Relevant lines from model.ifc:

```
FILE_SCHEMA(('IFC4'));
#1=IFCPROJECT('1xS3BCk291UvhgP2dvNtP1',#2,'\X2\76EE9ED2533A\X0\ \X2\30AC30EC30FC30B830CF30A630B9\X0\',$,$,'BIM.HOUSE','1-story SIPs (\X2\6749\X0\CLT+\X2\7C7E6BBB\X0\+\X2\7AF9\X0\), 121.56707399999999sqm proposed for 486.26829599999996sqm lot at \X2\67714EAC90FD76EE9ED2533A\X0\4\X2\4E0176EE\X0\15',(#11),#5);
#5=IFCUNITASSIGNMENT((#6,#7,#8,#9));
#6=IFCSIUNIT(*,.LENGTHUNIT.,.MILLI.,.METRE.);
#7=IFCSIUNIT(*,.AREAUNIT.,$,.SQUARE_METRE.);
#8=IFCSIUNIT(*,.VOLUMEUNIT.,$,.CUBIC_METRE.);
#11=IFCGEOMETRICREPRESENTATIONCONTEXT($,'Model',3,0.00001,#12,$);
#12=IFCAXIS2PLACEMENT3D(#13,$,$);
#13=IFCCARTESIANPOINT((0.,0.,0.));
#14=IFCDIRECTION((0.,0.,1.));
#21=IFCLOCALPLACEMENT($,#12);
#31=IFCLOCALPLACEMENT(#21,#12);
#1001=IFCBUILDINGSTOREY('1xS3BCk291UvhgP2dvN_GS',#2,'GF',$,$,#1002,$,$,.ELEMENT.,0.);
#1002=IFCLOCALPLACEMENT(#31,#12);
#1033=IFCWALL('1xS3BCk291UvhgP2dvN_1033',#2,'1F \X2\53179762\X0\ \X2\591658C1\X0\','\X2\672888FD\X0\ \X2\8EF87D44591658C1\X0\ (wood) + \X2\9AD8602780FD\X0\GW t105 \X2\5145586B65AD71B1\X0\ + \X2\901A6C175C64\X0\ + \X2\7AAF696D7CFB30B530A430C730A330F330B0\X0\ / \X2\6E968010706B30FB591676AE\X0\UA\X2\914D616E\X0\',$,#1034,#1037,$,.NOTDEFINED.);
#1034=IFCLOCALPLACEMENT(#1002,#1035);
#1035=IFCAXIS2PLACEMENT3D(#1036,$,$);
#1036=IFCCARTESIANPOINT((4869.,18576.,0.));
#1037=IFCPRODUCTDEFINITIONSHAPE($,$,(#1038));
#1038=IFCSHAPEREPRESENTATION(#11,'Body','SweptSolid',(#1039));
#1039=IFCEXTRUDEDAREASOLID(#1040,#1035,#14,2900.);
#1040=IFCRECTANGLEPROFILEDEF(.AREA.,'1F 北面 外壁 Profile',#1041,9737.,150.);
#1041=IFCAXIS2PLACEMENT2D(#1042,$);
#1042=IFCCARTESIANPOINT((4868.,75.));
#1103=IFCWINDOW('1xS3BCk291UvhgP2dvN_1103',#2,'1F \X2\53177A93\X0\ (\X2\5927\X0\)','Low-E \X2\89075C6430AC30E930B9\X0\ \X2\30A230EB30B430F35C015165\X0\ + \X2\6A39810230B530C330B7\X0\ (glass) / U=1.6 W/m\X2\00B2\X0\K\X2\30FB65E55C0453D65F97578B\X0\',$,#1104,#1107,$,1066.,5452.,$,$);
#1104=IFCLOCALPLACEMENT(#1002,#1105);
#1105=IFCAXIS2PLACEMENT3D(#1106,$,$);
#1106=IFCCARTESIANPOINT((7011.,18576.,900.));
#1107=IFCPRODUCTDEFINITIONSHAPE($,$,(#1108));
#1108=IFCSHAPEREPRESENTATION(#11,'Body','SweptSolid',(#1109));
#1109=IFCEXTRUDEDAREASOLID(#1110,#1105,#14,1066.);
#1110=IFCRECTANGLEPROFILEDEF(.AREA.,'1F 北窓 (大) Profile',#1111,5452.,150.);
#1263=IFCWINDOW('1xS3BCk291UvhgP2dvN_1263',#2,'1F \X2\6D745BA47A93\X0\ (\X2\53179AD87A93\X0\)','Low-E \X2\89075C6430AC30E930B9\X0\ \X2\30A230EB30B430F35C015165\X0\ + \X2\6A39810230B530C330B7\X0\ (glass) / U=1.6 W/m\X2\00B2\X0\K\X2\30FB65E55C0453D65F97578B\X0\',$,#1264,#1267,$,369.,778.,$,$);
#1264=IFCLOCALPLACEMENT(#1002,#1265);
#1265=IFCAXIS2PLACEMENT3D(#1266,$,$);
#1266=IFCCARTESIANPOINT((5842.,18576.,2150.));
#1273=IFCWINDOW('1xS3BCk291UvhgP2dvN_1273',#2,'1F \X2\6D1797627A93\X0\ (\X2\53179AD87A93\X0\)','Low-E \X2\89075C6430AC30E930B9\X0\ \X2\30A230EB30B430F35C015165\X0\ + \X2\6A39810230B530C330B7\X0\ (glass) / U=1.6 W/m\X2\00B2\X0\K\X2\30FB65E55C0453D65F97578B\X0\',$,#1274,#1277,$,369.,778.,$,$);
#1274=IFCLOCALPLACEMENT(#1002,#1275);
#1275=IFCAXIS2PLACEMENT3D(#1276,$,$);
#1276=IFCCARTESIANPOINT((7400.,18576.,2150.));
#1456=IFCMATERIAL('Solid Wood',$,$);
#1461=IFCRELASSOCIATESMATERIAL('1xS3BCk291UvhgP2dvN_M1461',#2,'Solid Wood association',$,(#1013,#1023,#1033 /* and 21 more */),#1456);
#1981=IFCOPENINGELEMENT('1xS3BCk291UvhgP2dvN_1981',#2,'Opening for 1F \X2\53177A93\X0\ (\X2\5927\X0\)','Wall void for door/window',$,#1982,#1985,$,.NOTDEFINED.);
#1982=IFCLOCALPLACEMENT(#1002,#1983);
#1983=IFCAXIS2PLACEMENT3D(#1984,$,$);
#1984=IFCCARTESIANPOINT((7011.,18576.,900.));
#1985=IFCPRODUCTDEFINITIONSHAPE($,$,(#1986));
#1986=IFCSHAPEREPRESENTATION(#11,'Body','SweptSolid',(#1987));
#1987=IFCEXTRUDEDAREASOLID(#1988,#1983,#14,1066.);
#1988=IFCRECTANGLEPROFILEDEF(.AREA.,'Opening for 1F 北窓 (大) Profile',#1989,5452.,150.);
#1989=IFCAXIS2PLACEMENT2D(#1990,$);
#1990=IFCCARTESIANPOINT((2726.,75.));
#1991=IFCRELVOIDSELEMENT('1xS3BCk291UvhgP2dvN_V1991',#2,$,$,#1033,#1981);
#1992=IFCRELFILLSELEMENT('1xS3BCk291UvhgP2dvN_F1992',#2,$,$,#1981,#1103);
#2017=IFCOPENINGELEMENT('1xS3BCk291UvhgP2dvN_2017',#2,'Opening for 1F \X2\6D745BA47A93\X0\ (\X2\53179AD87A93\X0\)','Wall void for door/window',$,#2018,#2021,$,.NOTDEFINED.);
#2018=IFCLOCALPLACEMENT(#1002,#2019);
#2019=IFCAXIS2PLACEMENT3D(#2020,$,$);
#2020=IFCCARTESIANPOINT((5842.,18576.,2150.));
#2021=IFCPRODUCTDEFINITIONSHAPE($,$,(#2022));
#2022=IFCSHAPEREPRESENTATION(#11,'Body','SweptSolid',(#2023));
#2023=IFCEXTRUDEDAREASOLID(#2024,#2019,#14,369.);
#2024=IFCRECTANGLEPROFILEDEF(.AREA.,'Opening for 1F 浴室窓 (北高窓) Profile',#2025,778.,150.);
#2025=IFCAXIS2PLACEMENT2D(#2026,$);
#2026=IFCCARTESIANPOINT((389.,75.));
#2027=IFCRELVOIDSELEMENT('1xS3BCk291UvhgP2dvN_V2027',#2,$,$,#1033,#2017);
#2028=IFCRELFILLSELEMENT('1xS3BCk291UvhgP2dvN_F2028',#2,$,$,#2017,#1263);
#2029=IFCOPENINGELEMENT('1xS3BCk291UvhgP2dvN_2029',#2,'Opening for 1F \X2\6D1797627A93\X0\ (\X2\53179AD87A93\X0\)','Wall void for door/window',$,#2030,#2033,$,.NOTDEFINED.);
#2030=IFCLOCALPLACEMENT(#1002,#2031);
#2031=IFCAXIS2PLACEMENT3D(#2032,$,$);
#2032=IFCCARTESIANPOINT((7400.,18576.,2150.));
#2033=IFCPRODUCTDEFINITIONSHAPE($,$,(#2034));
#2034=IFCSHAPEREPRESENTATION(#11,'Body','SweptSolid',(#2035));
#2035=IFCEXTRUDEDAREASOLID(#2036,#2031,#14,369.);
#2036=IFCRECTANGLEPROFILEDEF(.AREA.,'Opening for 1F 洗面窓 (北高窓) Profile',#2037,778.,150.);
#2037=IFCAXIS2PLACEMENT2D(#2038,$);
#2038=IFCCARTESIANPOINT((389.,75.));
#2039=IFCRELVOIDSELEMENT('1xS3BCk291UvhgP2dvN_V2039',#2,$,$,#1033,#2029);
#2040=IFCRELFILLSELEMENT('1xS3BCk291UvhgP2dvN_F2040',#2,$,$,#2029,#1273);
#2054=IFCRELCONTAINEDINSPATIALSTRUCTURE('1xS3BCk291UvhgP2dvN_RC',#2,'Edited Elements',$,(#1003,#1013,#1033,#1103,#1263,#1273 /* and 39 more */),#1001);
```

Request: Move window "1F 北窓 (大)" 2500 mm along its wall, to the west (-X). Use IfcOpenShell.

```python
import ifcopenshell
import ifcopenshell.api.geometry
import ifcopenshell.util.placement
import ifcopenshell.util.unit

model = ifcopenshell.open("model.ifc")
unit_scale = ifcopenshell.util.unit.calculate_unit_scale(model)

window = model.by_id(1103)
opening = window.FillsVoids[0].RelatingOpeningElement
wall = opening.VoidsElements[0].RelatingBuildingElement

wall_matrix = ifcopenshell.util.placement.get_local_placement(wall.ObjectPlacement)
shift = wall_matrix[:3, 0] * -2.5 / unit_scale
before = ifcopenshell.util.placement.get_local_placement(window.ObjectPlacement)[:3, 3].copy()

# The window is not placed relative to its opening, so move both.
for product in (opening, window):
    matrix = ifcopenshell.util.placement.get_local_placement(product.ObjectPlacement)
    matrix[:3, 3] += shift
    ifcopenshell.api.geometry.edit_object_placement(model, product=product, matrix=matrix, is_si=False)

after = ifcopenshell.util.placement.get_local_placement(window.ObjectPlacement)[:3, 3]
print("window moved by", (after - before).round(3) + 0.0)

model.write("model-out.ifc")
```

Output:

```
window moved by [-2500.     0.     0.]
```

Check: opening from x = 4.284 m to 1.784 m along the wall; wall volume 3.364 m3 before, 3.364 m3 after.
